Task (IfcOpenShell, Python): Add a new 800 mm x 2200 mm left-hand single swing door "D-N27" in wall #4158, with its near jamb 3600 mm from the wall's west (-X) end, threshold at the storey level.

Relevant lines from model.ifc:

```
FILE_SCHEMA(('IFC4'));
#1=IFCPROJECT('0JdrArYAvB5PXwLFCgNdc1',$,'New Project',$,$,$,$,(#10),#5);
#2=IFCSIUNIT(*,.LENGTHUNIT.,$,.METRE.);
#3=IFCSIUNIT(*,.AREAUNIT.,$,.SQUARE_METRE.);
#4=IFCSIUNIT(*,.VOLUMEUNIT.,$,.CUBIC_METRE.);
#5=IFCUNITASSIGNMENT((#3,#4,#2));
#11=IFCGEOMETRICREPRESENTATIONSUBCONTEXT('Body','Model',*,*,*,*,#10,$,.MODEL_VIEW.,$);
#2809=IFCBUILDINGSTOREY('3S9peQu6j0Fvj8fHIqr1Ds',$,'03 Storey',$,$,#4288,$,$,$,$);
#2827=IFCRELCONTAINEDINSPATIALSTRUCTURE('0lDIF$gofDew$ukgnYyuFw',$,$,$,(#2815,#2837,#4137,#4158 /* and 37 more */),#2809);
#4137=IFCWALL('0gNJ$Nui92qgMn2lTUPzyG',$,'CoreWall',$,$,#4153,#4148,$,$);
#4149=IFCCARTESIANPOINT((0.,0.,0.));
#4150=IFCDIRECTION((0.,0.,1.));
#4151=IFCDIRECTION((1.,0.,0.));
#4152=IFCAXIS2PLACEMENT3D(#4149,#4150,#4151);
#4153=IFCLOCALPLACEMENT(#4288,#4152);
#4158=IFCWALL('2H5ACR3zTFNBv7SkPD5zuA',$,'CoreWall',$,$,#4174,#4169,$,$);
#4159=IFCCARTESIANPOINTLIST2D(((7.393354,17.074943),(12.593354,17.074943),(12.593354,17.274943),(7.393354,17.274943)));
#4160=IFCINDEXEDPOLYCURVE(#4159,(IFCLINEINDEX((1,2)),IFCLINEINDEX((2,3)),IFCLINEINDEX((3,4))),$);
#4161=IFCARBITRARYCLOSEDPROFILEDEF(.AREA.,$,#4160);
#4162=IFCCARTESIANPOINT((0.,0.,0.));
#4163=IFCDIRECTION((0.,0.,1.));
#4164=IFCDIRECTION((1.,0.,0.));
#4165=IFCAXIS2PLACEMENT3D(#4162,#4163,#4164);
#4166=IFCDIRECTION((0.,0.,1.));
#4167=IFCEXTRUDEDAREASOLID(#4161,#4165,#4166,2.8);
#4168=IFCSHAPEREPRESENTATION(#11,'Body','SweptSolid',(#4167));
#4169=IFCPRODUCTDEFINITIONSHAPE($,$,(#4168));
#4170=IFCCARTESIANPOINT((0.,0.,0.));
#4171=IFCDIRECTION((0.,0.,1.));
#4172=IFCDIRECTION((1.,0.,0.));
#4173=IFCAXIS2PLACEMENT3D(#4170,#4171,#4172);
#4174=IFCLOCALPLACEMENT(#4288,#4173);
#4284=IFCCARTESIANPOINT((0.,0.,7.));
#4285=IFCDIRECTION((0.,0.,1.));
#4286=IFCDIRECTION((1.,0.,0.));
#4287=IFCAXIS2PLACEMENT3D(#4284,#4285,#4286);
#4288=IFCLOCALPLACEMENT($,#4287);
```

```python
import numpy as np
import ifcopenshell
import ifcopenshell.api.feature
import ifcopenshell.api.geometry
import ifcopenshell.api.root
import ifcopenshell.api.spatial
import ifcopenshell.geom
import ifcopenshell.util.element
import ifcopenshell.util.placement
import ifcopenshell.util.representation
import ifcopenshell.util.shape
import ifcopenshell.util.unit

model = ifcopenshell.open("model.ifc")
unit_scale = ifcopenshell.util.unit.calculate_unit_scale(model)
settings = ifcopenshell.geom.settings()


def volume(element):
    """Net volume in cubic metres, openings subtracted."""
    shape = ifcopenshell.geom.create_shape(settings, element)
    return ifcopenshell.util.shape.get_volume(shape.geometry)


wall = model.by_guid("2H5ACR3zTFNBv7SkPD5zuA")
storey = ifcopenshell.util.element.get_container(wall, ifc_class="IfcBuildingStorey")
context = ifcopenshell.util.representation.get_context(model, "Model", "Body", "MODEL_VIEW")
before = volume(wall)

width, height, from_end, sill = 0.8, 2.2, 3.6, 0.0  # metres

# The wall runs along its own X axis, and the end named is its -X end.
wall_shape = ifcopenshell.geom.create_shape(settings, wall)
x, y, z = ifcopenshell.util.shape.get_vertices(wall_shape.geometry).T
start = x.min() + from_end
face, thickness = float(y.min()), float(y.max() - y.min())
wall_matrix = ifcopenshell.util.placement.get_local_placement(wall.ObjectPlacement)
level = ifcopenshell.util.placement.get_local_placement(storey.ObjectPlacement)[2, 3]


def in_wall(x, y):
    """Placement at x, y metres in the wall's axes, at sill height."""
    matrix = wall_matrix.copy()
    matrix[:, 3] = wall_matrix @ np.array([x / unit_scale, y / unit_scale, 0.0, 1.0])
    matrix[2, 3] = level + sill / unit_scale
    return matrix


# Opening: a box that overshoots both wall faces by 50 mm.
opening = ifcopenshell.api.root.create_entity(model, ifc_class="IfcOpeningElement", predefined_type="OPENING")
box = ifcopenshell.api.geometry.add_wall_representation(
    model, context=context, length=width, height=height, thickness=thickness + 0.1
)
ifcopenshell.api.geometry.assign_representation(model, product=opening, representation=box)
ifcopenshell.api.geometry.edit_object_placement(model, product=opening, matrix=in_wall(start, face - 0.05), is_si=False)
ifcopenshell.api.feature.add_feature(model, feature=opening, element=wall)

door = ifcopenshell.api.root.create_entity(model, ifc_class="IfcDoor", name="D-N27", predefined_type="DOOR")
door.OverallWidth, door.OverallHeight = width / unit_scale, height / unit_scale
door.OperationType = "SINGLE_SWING_LEFT"
body = ifcopenshell.api.geometry.add_door_representation(
    model,
    context=context,
    overall_width=door.OverallWidth,
    overall_height=door.OverallHeight,
    operation_type="SINGLE_SWING_LEFT",
    lining_properties={"LiningDepth": thickness / unit_scale, "ThresholdDepth": thickness / unit_scale},
)
ifcopenshell.api.geometry.assign_representation(model, product=door, representation=body)
ifcopenshell.api.spatial.assign_container(model, products=[door], relating_structure=storey)
ifcopenshell.api.feature.add_filling(model, opening=opening, element=door)

# The lining spans the wall, so the door starts at the wall face.
ifcopenshell.api.geometry.edit_object_placement(model, product=door, matrix=in_wall(start, face), is_si=False)

after = volume(wall)

print(f"wall volume {before:.3f} -> {after:.3f} m3")

model.write("model_rev.ifc")
```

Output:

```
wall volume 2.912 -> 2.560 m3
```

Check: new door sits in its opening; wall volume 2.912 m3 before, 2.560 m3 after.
